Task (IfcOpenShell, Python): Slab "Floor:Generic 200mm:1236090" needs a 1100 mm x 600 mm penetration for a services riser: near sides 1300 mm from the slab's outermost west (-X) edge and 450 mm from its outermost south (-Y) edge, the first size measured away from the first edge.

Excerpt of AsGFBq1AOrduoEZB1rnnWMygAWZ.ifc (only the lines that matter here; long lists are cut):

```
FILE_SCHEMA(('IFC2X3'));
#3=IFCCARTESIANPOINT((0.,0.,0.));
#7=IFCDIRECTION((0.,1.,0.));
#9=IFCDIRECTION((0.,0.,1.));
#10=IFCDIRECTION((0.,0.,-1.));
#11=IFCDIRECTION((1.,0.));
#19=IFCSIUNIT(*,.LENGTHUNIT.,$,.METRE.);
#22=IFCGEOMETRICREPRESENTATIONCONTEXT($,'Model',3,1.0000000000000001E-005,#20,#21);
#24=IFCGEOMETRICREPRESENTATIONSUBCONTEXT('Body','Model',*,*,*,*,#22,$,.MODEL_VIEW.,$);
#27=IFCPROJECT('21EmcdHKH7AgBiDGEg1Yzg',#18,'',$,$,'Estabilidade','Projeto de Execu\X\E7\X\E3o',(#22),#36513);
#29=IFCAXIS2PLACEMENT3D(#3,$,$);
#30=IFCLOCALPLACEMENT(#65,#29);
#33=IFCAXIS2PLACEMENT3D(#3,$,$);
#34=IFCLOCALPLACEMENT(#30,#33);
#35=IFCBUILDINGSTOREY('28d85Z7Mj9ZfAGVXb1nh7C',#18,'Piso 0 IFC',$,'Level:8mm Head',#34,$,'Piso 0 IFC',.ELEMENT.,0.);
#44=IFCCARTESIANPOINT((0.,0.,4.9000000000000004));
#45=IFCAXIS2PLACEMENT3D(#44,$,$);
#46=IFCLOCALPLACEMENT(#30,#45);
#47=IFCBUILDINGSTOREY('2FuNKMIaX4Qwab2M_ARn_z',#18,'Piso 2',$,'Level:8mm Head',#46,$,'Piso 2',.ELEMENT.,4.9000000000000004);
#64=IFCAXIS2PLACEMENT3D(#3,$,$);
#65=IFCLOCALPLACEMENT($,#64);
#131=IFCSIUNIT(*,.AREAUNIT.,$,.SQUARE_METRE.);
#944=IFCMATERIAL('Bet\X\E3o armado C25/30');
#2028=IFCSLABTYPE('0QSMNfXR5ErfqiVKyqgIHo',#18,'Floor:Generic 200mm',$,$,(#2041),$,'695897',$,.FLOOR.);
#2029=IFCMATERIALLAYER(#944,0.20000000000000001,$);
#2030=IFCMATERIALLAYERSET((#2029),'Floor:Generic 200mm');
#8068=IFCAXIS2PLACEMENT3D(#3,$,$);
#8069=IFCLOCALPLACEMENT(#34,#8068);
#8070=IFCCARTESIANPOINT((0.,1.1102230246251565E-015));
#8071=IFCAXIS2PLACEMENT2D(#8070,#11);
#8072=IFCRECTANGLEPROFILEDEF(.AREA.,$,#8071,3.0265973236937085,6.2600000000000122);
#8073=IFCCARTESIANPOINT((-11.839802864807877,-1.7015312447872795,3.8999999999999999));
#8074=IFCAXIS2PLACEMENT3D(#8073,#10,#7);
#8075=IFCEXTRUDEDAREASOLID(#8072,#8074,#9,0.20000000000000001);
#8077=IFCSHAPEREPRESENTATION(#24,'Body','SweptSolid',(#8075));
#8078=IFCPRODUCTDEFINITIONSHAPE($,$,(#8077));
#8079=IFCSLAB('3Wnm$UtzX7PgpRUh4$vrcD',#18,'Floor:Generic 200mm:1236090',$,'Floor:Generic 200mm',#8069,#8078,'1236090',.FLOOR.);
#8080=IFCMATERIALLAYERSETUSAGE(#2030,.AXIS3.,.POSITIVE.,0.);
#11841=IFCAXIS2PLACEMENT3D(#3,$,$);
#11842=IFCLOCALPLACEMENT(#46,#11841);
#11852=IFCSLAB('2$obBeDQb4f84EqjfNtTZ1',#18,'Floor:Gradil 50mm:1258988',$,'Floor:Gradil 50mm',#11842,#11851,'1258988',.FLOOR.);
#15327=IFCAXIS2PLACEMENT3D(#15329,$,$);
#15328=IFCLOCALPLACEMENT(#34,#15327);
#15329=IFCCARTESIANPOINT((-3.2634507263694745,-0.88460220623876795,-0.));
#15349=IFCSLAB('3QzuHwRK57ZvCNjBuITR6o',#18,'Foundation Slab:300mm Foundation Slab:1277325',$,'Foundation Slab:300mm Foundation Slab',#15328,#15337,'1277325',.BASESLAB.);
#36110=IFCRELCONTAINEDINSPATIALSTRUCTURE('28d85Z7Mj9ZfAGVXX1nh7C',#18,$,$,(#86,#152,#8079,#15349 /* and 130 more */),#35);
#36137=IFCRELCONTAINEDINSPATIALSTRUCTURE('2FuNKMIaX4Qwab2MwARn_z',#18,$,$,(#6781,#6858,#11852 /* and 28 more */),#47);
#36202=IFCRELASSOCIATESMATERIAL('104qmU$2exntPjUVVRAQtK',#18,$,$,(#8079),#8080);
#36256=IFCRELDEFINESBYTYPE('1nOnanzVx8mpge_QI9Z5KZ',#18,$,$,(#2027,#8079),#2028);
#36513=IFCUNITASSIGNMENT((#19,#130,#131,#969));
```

```python
import numpy as np
import ifcopenshell
import ifcopenshell.api.feature
import ifcopenshell.api.geometry
import ifcopenshell.api.root
import ifcopenshell.geom
import ifcopenshell.util.placement
import ifcopenshell.util.representation
import ifcopenshell.util.shape
import ifcopenshell.util.unit

model = ifcopenshell.open("AsGFBq1AOrduoEZB1rnnWMygAWZ.ifc")
unit_scale = ifcopenshell.util.unit.calculate_unit_scale(model)
settings = ifcopenshell.geom.settings()


def volume(element):
    """Net volume in cubic metres, openings subtracted."""
    shape = ifcopenshell.geom.create_shape(settings, element)
    return ifcopenshell.util.shape.get_volume(shape.geometry)


slab = model.by_guid("3Wnm$UtzX7PgpRUh4$vrcD")
before = volume(slab)

# Extent in the slab's own axes, in metres. The edges named are its -X and -Y sides.
slab_shape = ifcopenshell.geom.create_shape(settings, slab)
vertices = ifcopenshell.util.shape.get_vertices(slab_shape.geometry)
x_min, y_min, bottom = vertices.min(axis=0)
top = vertices[:, 2].max()

opening = ifcopenshell.api.root.create_entity(model, ifc_class="IfcOpeningElement", name="Services riser opening")
context = ifcopenshell.util.representation.get_context(model, "Model", "Body", "MODEL_VIEW")
width, depth = 1.1, 0.6
outline = [(0.0, 0.0), (width, 0.0), (width, depth), (0.0, depth), (0.0, 0.0)]
# Overshoot both faces by 50 mm so the cut is clean.
shape = ifcopenshell.api.geometry.add_slab_representation(
    model, context=context, depth=top - bottom + 0.1, polyline=outline
)
ifcopenshell.api.geometry.assign_representation(model, product=opening, representation=shape)

matrix = ifcopenshell.util.placement.get_local_placement(slab.ObjectPlacement)
matrix[:, 3] = matrix @ np.append(np.array([x_min + 1.3, y_min + 0.45, bottom - 0.05]) / unit_scale, 1.0)
ifcopenshell.api.geometry.edit_object_placement(model, product=opening, matrix=matrix, is_si=False)
ifcopenshell.api.feature.add_feature(model, feature=opening, element=slab)

after = volume(slab)

print(f"slab volume {before:.3f} -> {after:.3f} m3")

model.write("AsGFBq1AOrduoEZB1rnnWMygAWZ_edited.ifc")
```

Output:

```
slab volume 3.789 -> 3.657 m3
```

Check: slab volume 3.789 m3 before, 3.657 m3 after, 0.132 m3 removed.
